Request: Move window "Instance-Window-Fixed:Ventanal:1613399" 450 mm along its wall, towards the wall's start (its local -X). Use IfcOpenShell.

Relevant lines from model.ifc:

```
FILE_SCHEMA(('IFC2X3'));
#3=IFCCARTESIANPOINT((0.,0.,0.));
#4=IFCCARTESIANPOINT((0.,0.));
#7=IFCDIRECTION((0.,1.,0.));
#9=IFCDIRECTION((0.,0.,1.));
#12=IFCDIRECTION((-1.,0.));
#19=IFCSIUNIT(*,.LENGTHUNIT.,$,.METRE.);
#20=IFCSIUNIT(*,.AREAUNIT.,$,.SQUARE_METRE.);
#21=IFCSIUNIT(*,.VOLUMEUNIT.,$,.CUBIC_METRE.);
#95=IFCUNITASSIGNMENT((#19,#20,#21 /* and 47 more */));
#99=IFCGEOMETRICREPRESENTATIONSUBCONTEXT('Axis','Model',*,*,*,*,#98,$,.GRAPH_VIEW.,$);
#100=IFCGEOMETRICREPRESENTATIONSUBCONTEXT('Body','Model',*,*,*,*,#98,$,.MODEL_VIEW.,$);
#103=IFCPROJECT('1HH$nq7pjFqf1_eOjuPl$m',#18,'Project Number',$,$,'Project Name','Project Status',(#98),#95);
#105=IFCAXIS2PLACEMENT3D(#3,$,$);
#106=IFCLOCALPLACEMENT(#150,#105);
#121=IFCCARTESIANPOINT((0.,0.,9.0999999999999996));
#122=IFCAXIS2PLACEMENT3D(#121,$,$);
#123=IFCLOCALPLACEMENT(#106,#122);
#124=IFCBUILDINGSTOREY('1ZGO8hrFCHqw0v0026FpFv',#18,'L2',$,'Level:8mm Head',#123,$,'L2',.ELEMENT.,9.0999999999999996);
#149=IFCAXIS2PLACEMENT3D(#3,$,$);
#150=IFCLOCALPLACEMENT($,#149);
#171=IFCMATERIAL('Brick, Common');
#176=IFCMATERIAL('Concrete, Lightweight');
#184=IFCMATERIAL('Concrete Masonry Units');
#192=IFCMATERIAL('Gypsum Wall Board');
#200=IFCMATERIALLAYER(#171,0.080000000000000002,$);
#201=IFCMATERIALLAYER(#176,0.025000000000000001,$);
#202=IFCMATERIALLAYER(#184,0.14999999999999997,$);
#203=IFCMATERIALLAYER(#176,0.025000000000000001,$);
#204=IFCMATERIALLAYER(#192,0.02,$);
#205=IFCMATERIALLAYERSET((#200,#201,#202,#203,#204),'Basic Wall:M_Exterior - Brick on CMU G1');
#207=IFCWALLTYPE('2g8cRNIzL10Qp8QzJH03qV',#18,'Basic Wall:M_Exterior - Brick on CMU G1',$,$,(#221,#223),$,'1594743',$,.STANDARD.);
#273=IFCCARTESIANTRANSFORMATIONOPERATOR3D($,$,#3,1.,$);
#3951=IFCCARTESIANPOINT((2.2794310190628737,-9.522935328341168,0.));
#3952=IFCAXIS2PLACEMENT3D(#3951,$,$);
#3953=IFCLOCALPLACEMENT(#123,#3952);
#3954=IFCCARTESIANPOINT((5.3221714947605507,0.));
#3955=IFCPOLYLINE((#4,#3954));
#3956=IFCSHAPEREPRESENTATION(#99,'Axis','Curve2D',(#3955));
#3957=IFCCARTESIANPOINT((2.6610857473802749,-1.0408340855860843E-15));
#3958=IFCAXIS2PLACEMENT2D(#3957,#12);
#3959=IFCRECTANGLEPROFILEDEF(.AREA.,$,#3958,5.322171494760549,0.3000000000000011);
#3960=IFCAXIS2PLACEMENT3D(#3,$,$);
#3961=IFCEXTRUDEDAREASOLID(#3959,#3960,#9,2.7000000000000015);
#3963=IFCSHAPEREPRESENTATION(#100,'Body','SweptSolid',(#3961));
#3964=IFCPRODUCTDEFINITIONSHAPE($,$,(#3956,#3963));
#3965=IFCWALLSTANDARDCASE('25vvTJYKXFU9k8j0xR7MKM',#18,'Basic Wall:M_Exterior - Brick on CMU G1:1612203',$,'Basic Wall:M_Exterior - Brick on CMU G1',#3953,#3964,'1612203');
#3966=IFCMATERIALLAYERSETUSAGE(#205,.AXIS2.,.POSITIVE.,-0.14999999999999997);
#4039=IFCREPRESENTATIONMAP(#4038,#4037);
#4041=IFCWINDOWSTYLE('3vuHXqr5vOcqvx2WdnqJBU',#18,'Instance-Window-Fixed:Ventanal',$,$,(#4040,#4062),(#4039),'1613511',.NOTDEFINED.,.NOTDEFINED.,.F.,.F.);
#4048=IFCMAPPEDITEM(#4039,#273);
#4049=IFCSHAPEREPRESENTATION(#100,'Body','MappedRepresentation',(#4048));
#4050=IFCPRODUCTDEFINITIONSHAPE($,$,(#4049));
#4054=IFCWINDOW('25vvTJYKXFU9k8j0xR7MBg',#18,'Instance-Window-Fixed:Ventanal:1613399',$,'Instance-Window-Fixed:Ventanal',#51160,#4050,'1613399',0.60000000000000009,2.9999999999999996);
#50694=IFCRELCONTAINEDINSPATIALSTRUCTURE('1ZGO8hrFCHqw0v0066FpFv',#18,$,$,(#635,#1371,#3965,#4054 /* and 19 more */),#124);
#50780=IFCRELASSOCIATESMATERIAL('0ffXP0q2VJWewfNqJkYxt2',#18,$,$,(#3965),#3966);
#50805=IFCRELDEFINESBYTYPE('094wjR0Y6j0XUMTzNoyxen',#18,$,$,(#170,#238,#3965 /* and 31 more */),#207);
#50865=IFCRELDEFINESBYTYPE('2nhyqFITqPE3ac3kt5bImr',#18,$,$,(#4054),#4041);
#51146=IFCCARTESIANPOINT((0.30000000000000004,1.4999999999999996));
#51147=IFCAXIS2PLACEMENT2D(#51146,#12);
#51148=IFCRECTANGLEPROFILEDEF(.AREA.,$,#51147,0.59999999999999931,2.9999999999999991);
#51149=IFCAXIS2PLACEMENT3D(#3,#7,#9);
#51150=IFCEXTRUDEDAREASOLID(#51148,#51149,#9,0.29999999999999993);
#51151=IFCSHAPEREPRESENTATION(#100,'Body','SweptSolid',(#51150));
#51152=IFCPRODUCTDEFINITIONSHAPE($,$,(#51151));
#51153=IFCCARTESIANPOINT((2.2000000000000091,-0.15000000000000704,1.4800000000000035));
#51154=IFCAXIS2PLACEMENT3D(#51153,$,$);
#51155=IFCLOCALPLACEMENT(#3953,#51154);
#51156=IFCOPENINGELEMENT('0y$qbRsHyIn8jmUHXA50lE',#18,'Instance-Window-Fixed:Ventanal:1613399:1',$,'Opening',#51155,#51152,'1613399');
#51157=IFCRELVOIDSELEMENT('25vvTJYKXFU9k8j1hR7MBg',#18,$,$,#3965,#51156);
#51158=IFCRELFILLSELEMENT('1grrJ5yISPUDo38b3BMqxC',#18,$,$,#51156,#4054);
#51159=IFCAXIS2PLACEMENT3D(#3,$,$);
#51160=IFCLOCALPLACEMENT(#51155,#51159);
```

```python
import ifcopenshell
import ifcopenshell.api.geometry
import ifcopenshell.util.placement
import ifcopenshell.util.unit

model = ifcopenshell.open("model.ifc")
unit_scale = ifcopenshell.util.unit.calculate_unit_scale(model)

window = model.by_guid("25vvTJYKXFU9k8j0xR7MBg")
opening = window.FillsVoids[0].RelatingOpeningElement
wall = opening.VoidsElements[0].RelatingBuildingElement

wall_matrix = ifcopenshell.util.placement.get_local_placement(wall.ObjectPlacement)
shift = wall_matrix[:3, 0] * -0.45 / unit_scale
before = ifcopenshell.util.placement.get_local_placement(window.ObjectPlacement)[:3, 3].copy()

# The window is placed relative to its opening, so it follows when the opening moves.
matrix = ifcopenshell.util.placement.get_local_placement(opening.ObjectPlacement)
matrix[:3, 3] += shift
ifcopenshell.api.geometry.edit_object_placement(
    model, product=opening, matrix=matrix, is_si=False, should_transform_children=True
)

after = ifcopenshell.util.placement.get_local_placement(window.ObjectPlacement)[:3, 3]
print("window moved by", (after - before).round(3) + 0.0)

model.write("model_edited.ifc")
```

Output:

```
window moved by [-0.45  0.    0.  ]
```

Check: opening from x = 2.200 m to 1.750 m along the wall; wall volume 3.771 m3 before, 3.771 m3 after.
